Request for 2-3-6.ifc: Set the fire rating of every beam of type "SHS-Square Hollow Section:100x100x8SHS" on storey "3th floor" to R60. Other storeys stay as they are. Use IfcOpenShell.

First a look at what the model holds.

```python
import ifcopenshell
import ifcopenshell.util.element

model = ifcopenshell.open("2-3-6.ifc")
print(model.schema)
storey = next(s for s in model.by_type("IfcBuildingStorey") if s.Name == "3th floor")
beams = [e for e in ifcopenshell.util.element.get_decomposition(storey) if e.is_a("IfcBeam")]
seen = {}
for e in beams:
    element_type = ifcopenshell.util.element.get_type(e)
    key = (element_type.Name if element_type != e and element_type else None, ifcopenshell.util.element.get_pset(e, "Pset_BeamCommon", "FireRating"))
    seen[key] = seen.get(key, 0) + 1
for (name, value), count in sorted(seen.items(), key=str):
    print(count, "x", name, "|", value)
```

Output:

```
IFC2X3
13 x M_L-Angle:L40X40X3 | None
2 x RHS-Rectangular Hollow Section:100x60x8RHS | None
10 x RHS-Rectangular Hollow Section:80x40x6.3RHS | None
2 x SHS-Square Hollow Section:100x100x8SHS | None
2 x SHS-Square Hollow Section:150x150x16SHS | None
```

```python
import ifcopenshell
import ifcopenshell.api.pset
import ifcopenshell.util.element

model = ifcopenshell.open("2-3-6.ifc")

storey = next(s for s in model.by_type("IfcBuildingStorey") if s.Name == "3th floor")
beams = [e for e in ifcopenshell.util.element.get_decomposition(storey) if e.is_a("IfcBeam")]

count = 0
for e in beams:
    element_type = ifcopenshell.util.element.get_type(e)
    if element_type in (None, e) or element_type.Name != "SHS-Square Hollow Section:100x100x8SHS":
        continue
    # add_pset returns the element's existing set when there is one.
    pset = ifcopenshell.api.pset.add_pset(model, product=e, name="Pset_BeamCommon")
    ifcopenshell.api.pset.edit_pset(model, pset=pset, properties={"FireRating": "R60"})
    count += 1

print(count, "beams updated")

model.write("2-3-6_updated.ifc")
```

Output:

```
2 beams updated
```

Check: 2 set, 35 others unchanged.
